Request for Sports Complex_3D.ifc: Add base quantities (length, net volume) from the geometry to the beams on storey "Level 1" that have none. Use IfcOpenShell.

First a look at what the model holds.

```python
import ifcopenshell
import ifcopenshell.util.element
import ifcopenshell.util.unit

model = ifcopenshell.open("Sports Complex_3D.ifc")
print(model.schema)
for unit_type in ("LENGTHUNIT", "AREAUNIT", "VOLUMEUNIT"):
    print(unit_type, ifcopenshell.util.unit.calculate_unit_scale(model, unit_type))
storey = next(s for s in model.by_type("IfcBuildingStorey") if s.Name == "Level 1")
beams = [e for e in ifcopenshell.util.element.get_decomposition(storey) if e.is_a("IfcBeam")]
for e in sorted(beams, key=lambda e: e.id()):
    print(e.id(), e.is_a(), e.Name, list(ifcopenshell.util.element.get_psets(e, qtos_only=True)), sep=" | ")
```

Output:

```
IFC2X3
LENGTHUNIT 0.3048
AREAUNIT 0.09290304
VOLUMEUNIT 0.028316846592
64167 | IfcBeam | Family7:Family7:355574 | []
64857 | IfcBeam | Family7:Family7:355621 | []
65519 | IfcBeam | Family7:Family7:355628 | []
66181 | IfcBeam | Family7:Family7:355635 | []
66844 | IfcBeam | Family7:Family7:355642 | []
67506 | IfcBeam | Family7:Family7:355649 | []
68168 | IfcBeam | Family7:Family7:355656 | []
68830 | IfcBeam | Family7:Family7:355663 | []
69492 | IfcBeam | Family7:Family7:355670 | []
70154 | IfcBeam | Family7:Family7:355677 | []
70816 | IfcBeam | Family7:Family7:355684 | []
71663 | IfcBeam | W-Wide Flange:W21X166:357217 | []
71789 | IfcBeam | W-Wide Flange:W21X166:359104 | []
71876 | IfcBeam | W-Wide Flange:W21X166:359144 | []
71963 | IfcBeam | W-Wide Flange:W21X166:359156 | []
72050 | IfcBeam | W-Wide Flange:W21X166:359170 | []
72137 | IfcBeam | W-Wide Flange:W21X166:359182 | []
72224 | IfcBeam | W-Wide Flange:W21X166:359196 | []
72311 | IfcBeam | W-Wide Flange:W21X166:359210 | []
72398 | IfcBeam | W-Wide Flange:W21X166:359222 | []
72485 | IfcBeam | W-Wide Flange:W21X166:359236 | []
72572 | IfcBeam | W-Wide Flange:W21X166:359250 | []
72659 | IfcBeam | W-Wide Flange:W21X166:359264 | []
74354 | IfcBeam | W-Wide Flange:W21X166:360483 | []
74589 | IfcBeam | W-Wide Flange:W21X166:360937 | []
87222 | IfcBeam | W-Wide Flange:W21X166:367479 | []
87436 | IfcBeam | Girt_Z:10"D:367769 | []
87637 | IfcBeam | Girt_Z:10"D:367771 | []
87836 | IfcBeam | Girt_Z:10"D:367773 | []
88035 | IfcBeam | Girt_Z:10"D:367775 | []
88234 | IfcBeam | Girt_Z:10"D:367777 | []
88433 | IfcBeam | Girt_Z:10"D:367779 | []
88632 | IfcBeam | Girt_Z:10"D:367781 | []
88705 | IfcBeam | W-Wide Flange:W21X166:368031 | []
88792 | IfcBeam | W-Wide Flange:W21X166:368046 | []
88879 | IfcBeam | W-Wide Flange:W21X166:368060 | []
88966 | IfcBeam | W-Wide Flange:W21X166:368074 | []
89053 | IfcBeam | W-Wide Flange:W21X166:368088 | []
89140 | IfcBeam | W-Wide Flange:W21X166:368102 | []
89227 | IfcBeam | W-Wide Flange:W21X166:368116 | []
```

```python
import ifcopenshell
import ifcopenshell.api.pset
import ifcopenshell.geom
import ifcopenshell.util.element
import ifcopenshell.util.shape
import ifcopenshell.util.unit

model = ifcopenshell.open("Sports Complex_3D.ifc")
unit_scale = ifcopenshell.util.unit.calculate_unit_scale(model)
volume_scale = ifcopenshell.util.unit.calculate_unit_scale(model, "VOLUMEUNIT")
settings = ifcopenshell.geom.settings()

storey = next(s for s in model.by_type("IfcBuildingStorey") if s.Name == "Level 1")
beams = [e for e in ifcopenshell.util.element.get_decomposition(storey) if e.is_a("IfcBeam")]

for e in sorted(beams, key=lambda e: e.id()):
    if ifcopenshell.util.element.get_psets(e, qtos_only=True, should_inherit=False):
        continue
    # Geometry comes back in metres, in the element's own axes.
    shape = ifcopenshell.geom.create_shape(settings, e)
    values = {
        "Length": ifcopenshell.util.shape.get_max_xyz(shape.geometry) / unit_scale,
        "NetVolume": ifcopenshell.util.shape.get_volume(shape.geometry) / volume_scale,
    }
    qto = ifcopenshell.api.pset.add_qto(model, product=e, name="BaseQuantities")
    ifcopenshell.api.pset.edit_qto(model, qto=qto, properties=values)
    print(e.id(), {k: round(v, 3) for k, v in values.items()})

model.write("Sports Complex_3D-out.ifc")
```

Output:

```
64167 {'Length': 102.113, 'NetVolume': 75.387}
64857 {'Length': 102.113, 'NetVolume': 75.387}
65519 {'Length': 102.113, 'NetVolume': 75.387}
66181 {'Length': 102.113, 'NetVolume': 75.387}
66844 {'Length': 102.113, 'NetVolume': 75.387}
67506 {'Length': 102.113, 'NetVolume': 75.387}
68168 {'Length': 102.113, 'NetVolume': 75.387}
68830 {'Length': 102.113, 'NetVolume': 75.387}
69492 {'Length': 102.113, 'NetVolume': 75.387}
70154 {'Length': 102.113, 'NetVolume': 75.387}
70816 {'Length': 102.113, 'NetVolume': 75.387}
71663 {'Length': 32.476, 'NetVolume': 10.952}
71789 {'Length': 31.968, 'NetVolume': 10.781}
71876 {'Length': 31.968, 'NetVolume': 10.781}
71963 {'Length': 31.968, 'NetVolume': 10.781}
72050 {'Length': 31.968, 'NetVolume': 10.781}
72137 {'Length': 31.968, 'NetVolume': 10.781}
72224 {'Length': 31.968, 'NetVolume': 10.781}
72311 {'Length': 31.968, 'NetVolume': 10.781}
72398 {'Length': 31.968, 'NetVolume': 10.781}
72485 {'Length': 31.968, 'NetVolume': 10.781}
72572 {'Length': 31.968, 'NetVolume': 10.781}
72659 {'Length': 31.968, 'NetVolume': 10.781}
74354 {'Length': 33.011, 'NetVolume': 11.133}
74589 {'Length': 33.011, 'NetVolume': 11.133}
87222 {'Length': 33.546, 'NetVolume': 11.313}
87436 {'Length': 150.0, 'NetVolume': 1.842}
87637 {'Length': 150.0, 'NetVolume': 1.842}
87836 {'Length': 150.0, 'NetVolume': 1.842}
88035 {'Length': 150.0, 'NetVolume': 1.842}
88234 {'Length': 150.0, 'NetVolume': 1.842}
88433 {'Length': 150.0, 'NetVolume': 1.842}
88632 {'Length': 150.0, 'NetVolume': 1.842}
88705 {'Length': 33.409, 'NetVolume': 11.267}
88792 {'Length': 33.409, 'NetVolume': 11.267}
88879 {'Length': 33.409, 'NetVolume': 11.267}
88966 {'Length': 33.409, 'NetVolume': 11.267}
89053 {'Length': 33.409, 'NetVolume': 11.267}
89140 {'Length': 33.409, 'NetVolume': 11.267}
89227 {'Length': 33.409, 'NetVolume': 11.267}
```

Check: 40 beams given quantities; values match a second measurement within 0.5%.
